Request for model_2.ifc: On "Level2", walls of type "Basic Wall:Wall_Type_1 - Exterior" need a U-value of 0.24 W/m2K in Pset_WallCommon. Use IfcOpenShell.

First a look at what the model holds.

```python
import ifcopenshell
import ifcopenshell.util.element

model = ifcopenshell.open("model_2.ifc")
print(model.schema)
storey = next(s for s in model.by_type("IfcBuildingStorey") if s.Name == "Level2")
walls = [e for e in ifcopenshell.util.element.get_decomposition(storey) if e.is_a("IfcWall")]
seen = {}
for e in walls:
    element_type = ifcopenshell.util.element.get_type(e)
    key = (element_type.Name if element_type != e and element_type else None, ifcopenshell.util.element.get_pset(e, "Pset_WallCommon", "ThermalTransmittance"))
    seen[key] = seen.get(key, 0) + 1
for (name, value), count in sorted(seen.items(), key=str):
    print(count, "x", name, "|", value)
```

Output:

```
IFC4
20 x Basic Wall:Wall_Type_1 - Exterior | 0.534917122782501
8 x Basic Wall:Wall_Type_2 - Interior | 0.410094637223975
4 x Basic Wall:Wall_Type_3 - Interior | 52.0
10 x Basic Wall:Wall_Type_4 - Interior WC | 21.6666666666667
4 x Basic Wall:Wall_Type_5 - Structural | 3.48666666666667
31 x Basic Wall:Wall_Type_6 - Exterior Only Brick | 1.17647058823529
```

```python
import ifcopenshell
import ifcopenshell.api.pset
import ifcopenshell.util.element

model = ifcopenshell.open("model_2.ifc")

storey = next(s for s in model.by_type("IfcBuildingStorey") if s.Name == "Level2")
walls = [e for e in ifcopenshell.util.element.get_decomposition(storey) if e.is_a("IfcWall")]

count = 0
for e in walls:
    element_type = ifcopenshell.util.element.get_type(e)
    if element_type in (None, e) or element_type.Name != "Basic Wall:Wall_Type_1 - Exterior":
        continue
    # add_pset returns the element's existing set when there is one.
    pset = ifcopenshell.api.pset.add_pset(model, product=e, name="Pset_WallCommon")
    ifcopenshell.api.pset.edit_pset(model, pset=pset, properties={"ThermalTransmittance": 0.24})
    count += 1

print(count, "walls updated")

model.write("model_2_rev.ifc")
```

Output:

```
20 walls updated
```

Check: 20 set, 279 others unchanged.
